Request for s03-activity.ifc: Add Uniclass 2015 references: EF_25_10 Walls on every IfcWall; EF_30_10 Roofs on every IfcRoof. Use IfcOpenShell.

First a look at what the model holds.

```python
import ifcopenshell

model = ifcopenshell.open("s03-activity.ifc")
print(model.schema)
print("classifications:", [c.Name for c in model.by_type("IfcClassification")])
for ifc_class in ("IfcDoor", "IfcRoof", "IfcStair", "IfcWall", "IfcWindow"):
    print(ifc_class, len(model.by_type(ifc_class)))
```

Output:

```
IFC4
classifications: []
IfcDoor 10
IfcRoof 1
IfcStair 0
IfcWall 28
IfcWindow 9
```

```python
import ifcopenshell
import ifcopenshell.api.classification

model = ifcopenshell.open("s03-activity.ifc")

system = ifcopenshell.api.classification.add_classification(model, classification="Uniclass 2015")

codes = {
    "IfcWall": ("EF_25_10", "Walls"),
    "IfcRoof": ("EF_30_10", "Roofs"),
}
for ifc_class, (code, name) in codes.items():
    products = model.by_type(ifc_class)
    ifcopenshell.api.classification.add_reference(
        model, products=products, classification=system, identification=code, name=name
    )
    print(code, len(products))

model.write("s03-activity_updated.ifc")
```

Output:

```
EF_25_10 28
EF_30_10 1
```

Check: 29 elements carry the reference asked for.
